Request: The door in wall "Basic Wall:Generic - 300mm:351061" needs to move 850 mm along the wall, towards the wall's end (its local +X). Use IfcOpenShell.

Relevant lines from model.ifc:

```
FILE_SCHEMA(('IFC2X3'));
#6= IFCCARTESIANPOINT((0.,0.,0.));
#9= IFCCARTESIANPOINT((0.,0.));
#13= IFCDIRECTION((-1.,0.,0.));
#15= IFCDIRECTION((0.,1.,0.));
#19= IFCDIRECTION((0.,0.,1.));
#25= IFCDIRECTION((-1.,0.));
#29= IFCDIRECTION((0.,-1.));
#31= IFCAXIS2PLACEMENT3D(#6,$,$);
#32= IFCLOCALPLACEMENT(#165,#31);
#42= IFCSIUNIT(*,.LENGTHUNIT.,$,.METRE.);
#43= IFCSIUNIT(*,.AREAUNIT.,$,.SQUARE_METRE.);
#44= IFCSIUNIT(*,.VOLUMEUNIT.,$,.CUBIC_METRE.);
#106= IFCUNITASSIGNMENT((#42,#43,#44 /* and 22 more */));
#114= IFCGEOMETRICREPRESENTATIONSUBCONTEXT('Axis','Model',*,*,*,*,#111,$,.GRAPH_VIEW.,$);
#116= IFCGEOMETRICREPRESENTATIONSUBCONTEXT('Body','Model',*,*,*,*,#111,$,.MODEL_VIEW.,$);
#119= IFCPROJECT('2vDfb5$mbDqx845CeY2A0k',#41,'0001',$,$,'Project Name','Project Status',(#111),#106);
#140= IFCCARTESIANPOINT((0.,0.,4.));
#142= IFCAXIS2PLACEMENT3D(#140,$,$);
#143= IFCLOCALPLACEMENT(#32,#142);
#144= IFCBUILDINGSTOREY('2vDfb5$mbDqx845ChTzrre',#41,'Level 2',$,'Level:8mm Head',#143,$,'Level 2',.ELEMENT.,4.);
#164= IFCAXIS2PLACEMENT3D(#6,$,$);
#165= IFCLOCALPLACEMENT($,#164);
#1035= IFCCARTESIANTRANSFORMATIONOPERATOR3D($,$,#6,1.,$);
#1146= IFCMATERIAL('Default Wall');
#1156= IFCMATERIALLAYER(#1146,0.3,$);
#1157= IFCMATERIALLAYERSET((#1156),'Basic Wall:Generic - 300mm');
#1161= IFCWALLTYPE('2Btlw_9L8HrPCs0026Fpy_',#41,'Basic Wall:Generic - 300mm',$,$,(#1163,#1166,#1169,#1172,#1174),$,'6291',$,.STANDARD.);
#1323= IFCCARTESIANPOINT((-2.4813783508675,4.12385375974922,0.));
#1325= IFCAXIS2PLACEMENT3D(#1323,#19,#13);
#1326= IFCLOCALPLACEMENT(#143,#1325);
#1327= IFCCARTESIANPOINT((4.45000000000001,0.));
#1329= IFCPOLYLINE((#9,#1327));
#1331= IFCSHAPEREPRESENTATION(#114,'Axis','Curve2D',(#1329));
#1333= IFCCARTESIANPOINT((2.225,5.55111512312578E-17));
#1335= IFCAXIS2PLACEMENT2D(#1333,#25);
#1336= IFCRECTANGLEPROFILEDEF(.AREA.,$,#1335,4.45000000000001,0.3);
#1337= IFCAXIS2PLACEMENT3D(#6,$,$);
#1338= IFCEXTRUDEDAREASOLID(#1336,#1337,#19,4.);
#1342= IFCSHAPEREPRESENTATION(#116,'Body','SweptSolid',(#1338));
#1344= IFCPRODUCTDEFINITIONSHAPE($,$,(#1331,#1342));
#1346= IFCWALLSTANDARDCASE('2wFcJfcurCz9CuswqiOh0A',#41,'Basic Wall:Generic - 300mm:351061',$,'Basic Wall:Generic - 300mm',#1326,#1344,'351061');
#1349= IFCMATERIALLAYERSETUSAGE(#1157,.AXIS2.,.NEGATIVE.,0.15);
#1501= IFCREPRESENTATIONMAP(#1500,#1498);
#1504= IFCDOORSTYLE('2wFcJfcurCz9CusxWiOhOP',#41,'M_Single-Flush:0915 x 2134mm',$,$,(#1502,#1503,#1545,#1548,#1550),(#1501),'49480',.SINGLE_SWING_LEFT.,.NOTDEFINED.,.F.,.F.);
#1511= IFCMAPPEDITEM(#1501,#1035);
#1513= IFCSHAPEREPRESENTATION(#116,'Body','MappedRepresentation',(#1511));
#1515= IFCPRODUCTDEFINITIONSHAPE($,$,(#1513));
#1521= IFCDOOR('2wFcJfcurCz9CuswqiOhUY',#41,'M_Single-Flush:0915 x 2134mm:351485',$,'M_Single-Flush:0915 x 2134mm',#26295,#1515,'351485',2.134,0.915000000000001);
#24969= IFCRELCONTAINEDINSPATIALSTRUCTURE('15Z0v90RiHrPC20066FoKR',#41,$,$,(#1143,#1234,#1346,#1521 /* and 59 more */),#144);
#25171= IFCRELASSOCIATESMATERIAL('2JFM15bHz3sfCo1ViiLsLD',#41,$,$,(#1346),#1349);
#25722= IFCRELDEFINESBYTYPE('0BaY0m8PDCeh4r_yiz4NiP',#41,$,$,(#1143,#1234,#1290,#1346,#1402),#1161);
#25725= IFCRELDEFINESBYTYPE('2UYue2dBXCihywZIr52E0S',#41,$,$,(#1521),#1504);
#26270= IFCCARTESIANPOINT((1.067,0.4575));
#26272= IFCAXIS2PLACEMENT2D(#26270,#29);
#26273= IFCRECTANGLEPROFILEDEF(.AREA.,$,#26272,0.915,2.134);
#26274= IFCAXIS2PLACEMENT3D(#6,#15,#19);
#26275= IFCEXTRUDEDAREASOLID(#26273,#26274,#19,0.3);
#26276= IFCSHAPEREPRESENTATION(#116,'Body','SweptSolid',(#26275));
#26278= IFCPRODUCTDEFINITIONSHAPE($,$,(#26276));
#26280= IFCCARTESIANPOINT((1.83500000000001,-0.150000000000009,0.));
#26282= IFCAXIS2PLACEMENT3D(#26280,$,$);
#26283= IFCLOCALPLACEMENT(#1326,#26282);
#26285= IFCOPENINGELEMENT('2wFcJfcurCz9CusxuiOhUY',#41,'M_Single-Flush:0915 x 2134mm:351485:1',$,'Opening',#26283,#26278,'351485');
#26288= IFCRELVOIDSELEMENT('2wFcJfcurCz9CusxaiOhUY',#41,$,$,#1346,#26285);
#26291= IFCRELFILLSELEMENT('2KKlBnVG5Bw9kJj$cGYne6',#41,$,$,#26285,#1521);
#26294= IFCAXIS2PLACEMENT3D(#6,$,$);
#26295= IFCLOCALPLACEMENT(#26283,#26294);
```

```python
import ifcopenshell
import ifcopenshell.api.geometry
import ifcopenshell.util.placement
import ifcopenshell.util.unit

model = ifcopenshell.open("model.ifc")
unit_scale = ifcopenshell.util.unit.calculate_unit_scale(model)

door = model.by_id(1521)
opening = door.FillsVoids[0].RelatingOpeningElement
wall = opening.VoidsElements[0].RelatingBuildingElement

wall_matrix = ifcopenshell.util.placement.get_local_placement(wall.ObjectPlacement)
shift = wall_matrix[:3, 0] * 0.85 / unit_scale
before = ifcopenshell.util.placement.get_local_placement(door.ObjectPlacement)[:3, 3].copy()

# The door is placed relative to its opening, so it follows when the opening moves.
matrix = ifcopenshell.util.placement.get_local_placement(opening.ObjectPlacement)
matrix[:3, 3] += shift
ifcopenshell.api.geometry.edit_object_placement(
    model, product=opening, matrix=matrix, is_si=False, should_transform_children=True
)

after = ifcopenshell.util.placement.get_local_placement(door.ObjectPlacement)[:3, 3]
print("door moved by", (after - before).round(3) + 0.0)

model.write("model_v2.ifc")
```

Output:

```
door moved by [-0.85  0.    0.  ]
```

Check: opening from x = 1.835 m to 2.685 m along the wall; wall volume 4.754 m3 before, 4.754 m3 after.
